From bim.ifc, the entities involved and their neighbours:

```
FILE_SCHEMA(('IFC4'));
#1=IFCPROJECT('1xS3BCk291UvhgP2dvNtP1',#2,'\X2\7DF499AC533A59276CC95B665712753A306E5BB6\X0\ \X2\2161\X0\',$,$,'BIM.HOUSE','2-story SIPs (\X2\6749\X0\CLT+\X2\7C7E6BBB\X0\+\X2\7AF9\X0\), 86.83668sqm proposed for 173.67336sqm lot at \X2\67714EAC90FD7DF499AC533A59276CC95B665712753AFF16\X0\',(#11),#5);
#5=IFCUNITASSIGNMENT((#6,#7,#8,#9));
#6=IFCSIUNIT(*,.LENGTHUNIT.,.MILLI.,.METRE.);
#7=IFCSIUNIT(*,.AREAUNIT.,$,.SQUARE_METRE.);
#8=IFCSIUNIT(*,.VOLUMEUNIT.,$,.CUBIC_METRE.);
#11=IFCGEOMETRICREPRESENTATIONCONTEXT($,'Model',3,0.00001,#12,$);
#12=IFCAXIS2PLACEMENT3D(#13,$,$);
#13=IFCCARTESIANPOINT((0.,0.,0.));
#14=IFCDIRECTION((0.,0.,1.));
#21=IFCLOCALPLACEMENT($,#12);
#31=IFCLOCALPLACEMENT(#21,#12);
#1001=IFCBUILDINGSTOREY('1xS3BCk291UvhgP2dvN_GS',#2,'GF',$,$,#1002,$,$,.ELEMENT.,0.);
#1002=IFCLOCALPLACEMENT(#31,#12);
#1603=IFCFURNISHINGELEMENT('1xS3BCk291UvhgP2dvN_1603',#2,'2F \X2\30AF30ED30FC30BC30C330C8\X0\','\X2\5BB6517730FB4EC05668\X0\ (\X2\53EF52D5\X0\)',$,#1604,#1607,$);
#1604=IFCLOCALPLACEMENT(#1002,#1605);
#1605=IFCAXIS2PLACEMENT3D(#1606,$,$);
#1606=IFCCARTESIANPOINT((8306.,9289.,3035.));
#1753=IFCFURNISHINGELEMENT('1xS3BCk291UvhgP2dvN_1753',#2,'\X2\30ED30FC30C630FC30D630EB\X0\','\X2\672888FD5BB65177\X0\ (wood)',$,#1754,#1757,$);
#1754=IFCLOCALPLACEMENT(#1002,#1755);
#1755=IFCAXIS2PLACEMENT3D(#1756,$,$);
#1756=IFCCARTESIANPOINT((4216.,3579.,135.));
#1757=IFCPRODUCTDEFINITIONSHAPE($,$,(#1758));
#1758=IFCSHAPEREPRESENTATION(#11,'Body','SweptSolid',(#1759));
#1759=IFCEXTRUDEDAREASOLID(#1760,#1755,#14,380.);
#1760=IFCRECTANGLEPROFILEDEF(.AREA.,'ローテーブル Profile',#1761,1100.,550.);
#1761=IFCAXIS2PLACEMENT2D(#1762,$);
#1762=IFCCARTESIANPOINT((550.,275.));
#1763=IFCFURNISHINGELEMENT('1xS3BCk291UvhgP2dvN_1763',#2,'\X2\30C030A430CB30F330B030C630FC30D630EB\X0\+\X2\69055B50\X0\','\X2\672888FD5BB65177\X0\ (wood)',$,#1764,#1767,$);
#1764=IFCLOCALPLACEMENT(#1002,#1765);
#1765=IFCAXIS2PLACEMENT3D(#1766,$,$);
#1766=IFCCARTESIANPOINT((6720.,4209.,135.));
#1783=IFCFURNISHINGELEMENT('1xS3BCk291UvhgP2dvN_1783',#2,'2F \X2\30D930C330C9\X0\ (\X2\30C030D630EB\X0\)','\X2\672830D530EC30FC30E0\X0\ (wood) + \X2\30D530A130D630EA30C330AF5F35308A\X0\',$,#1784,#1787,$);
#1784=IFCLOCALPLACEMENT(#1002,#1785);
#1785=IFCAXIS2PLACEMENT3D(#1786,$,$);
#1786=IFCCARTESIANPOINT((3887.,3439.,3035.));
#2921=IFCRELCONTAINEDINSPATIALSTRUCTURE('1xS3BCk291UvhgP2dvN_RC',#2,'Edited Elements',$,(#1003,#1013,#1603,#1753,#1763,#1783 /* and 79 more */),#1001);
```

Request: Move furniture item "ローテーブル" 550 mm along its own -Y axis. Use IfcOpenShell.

```python
import ifcopenshell
import ifcopenshell.api.geometry
import ifcopenshell.util.placement

model = ifcopenshell.open("bim.ifc")

item = model.by_guid("1xS3BCk291UvhgP2dvN_1753")
matrix = ifcopenshell.util.placement.get_local_placement(item.ObjectPlacement)
matrix[:3, 3] -= matrix[:3, 1] * 550.0
ifcopenshell.api.geometry.edit_object_placement(model, product=item, matrix=matrix, is_si=False)

print(ifcopenshell.util.placement.get_local_placement(item.ObjectPlacement).round(3) + 0.0)

model.write("bim-out.ifc")
```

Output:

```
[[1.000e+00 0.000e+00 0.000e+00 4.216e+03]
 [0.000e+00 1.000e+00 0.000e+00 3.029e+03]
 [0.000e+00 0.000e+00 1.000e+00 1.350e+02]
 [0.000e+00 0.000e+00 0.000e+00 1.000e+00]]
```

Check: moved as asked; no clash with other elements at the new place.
